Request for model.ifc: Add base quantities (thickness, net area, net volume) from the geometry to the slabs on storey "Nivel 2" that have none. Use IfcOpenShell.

First a look at what the model holds.

```python
import ifcopenshell
import ifcopenshell.util.element
import ifcopenshell.util.unit

model = ifcopenshell.open("model.ifc")
print(model.schema)
for unit_type in ("LENGTHUNIT", "AREAUNIT", "VOLUMEUNIT"):
    print(unit_type, ifcopenshell.util.unit.calculate_unit_scale(model, unit_type))
storey = next(s for s in model.by_type("IfcBuildingStorey") if s.Name == "Nivel 2")
slabs = [e for e in ifcopenshell.util.element.get_decomposition(storey) if e.is_a("IfcSlab")]
for e in sorted(slabs, key=lambda e: e.id()):
    print(e.id(), e.is_a(), e.Name, list(ifcopenshell.util.element.get_psets(e, qtos_only=True)), sep=" | ")
```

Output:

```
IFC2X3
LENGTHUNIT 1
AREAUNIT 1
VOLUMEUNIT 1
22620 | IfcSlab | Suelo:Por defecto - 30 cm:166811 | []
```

```python
import ifcopenshell
import ifcopenshell.api.pset
import ifcopenshell.geom
import ifcopenshell.util.element
import ifcopenshell.util.shape
import ifcopenshell.util.unit

model = ifcopenshell.open("model.ifc")
unit_scale = ifcopenshell.util.unit.calculate_unit_scale(model)
area_scale = ifcopenshell.util.unit.calculate_unit_scale(model, "AREAUNIT")
volume_scale = ifcopenshell.util.unit.calculate_unit_scale(model, "VOLUMEUNIT")
settings = ifcopenshell.geom.settings()

storey = next(s for s in model.by_type("IfcBuildingStorey") if s.Name == "Nivel 2")
slabs = [e for e in ifcopenshell.util.element.get_decomposition(storey) if e.is_a("IfcSlab")]

for e in sorted(slabs, key=lambda e: e.id()):
    if ifcopenshell.util.element.get_psets(e, qtos_only=True, should_inherit=False):
        continue
    # Geometry comes back in metres, in the element's own axes.
    shape = ifcopenshell.geom.create_shape(settings, e)
    values = {
        "Width": ifcopenshell.util.shape.get_z(shape.geometry) / unit_scale,
        "NetArea": ifcopenshell.util.shape.get_footprint_area(shape.geometry) / area_scale,
        "NetVolume": ifcopenshell.util.shape.get_volume(shape.geometry) / volume_scale,
    }
    qto = ifcopenshell.api.pset.add_qto(model, product=e, name="BaseQuantities")
    ifcopenshell.api.pset.edit_qto(model, qto=qto, properties=values)
    print(e.id(), {k: round(v, 3) for k, v in values.items()})

model.write("model_v2.ifc")
```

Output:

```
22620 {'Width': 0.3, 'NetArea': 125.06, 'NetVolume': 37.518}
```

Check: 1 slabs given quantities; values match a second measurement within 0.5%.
